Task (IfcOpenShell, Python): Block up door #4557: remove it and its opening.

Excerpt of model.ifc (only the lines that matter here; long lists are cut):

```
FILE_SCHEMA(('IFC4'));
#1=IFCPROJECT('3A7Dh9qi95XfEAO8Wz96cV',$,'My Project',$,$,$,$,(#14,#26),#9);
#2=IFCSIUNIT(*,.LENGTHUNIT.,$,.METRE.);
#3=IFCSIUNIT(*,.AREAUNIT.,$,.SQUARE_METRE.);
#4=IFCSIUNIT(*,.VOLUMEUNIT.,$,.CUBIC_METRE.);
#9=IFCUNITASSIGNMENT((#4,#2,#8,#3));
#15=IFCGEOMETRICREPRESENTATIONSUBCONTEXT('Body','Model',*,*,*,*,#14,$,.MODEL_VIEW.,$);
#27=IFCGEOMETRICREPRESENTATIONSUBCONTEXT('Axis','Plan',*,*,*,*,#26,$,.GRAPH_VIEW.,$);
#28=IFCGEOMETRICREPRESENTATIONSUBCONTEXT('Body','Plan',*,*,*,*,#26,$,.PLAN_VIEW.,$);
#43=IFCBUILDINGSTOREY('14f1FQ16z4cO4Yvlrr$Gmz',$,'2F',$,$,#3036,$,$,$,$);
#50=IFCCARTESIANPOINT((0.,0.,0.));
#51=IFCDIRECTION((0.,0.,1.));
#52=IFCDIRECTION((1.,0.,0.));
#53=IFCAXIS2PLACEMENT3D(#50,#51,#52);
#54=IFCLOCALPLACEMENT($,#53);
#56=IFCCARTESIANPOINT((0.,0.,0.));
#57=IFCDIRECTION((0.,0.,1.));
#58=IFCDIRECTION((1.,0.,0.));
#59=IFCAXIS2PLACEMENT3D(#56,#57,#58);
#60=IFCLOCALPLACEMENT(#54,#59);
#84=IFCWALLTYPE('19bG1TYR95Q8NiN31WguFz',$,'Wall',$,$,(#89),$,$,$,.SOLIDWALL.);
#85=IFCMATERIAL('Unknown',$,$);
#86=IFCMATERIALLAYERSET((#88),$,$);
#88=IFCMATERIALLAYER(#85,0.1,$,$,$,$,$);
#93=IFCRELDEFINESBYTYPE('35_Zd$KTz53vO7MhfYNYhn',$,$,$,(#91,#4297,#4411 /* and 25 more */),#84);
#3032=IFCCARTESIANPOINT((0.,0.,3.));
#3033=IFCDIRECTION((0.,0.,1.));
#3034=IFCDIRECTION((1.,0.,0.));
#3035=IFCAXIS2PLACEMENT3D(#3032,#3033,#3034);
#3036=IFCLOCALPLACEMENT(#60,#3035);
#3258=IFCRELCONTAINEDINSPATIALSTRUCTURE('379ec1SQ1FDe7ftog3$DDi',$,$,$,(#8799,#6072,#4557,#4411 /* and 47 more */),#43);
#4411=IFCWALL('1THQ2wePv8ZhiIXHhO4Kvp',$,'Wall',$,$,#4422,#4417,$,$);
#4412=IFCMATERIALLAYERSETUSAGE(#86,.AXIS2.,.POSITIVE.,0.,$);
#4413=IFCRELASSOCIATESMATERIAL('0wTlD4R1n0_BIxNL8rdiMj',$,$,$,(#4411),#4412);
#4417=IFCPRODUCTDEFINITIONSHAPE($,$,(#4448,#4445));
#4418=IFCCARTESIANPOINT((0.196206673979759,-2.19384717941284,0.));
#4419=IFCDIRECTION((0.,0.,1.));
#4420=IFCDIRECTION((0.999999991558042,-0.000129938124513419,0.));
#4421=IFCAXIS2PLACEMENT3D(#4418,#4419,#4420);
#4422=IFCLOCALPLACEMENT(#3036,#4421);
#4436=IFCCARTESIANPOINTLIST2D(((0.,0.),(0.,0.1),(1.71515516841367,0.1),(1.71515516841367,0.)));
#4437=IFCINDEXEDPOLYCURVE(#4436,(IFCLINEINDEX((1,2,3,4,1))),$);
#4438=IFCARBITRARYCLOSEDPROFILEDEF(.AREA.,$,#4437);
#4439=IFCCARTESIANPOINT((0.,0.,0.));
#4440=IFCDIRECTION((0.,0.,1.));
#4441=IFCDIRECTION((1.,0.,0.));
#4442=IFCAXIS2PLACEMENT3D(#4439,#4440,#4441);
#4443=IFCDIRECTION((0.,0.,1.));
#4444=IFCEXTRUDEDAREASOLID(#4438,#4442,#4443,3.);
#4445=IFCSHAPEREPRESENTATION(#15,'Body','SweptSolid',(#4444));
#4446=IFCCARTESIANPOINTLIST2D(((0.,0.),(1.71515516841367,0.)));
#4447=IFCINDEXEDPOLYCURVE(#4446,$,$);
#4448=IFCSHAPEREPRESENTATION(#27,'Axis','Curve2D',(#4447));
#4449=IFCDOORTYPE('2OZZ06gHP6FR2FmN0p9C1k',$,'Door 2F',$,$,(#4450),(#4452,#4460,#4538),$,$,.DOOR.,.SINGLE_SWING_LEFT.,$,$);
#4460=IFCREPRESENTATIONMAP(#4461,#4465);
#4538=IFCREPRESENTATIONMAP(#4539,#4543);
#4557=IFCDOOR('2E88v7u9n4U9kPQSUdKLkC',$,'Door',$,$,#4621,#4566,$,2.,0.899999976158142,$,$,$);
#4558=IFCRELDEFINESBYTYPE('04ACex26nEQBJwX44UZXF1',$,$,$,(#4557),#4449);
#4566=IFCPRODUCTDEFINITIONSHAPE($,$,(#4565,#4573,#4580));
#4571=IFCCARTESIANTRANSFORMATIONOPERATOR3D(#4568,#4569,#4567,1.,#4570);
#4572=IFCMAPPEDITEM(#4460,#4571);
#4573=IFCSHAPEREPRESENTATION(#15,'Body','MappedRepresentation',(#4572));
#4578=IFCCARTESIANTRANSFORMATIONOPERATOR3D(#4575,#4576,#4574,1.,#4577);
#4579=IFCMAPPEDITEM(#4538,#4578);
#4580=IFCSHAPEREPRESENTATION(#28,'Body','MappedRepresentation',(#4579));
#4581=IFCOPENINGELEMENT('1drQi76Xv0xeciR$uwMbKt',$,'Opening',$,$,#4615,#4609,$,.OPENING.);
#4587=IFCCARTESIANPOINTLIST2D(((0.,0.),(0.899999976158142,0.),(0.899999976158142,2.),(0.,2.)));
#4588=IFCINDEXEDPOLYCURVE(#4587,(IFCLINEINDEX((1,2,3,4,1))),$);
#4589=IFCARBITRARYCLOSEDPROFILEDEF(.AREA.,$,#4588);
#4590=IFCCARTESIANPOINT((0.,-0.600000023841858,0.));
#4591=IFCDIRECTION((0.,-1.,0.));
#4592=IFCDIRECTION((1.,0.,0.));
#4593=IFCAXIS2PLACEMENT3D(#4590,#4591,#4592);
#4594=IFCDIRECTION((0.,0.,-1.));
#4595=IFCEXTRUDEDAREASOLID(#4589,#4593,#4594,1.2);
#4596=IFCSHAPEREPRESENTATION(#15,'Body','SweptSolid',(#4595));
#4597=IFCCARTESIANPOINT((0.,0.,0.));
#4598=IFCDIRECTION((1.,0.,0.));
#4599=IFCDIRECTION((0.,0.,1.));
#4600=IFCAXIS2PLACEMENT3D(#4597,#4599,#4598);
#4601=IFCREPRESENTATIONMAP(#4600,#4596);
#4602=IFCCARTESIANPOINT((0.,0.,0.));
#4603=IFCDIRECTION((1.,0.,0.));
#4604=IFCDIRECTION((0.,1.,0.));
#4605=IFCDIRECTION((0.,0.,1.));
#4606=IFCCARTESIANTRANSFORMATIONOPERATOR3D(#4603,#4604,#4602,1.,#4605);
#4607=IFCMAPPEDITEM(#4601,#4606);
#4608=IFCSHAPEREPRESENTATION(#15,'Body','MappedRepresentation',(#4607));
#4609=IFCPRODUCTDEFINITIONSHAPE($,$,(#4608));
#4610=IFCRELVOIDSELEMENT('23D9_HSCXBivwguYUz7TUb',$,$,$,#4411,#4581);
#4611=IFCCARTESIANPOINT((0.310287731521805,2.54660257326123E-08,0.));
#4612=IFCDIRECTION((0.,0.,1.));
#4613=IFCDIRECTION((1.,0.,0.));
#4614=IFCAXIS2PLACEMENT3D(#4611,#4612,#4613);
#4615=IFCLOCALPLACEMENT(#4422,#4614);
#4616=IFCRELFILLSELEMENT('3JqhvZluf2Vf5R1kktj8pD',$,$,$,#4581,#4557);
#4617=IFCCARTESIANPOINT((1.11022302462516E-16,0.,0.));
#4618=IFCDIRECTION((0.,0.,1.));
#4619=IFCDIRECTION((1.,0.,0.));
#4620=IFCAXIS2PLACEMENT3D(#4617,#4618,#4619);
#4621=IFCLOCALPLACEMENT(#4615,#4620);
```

```python
import ifcopenshell
import ifcopenshell.api.feature
import ifcopenshell.api.root
import ifcopenshell.geom
import ifcopenshell.util.shape

model = ifcopenshell.open("model.ifc")
settings = ifcopenshell.geom.settings()


def volume(element):
    """Net volume in cubic metres, openings subtracted."""
    shape = ifcopenshell.geom.create_shape(settings, element)
    return ifcopenshell.util.shape.get_volume(shape.geometry)


door = model.by_id(4557)
opening = door.FillsVoids[0].RelatingOpeningElement
wall = opening.VoidsElements[0].RelatingBuildingElement
before = volume(wall)

ifcopenshell.api.root.remove_product(model, product=door)
ifcopenshell.api.feature.remove_feature(model, feature=opening)

after = volume(wall)

print(f"wall volume {before:.3f} -> {after:.3f} m3")

model.write("model-out.ifc")
```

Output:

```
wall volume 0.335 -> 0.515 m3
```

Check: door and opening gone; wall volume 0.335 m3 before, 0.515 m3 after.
